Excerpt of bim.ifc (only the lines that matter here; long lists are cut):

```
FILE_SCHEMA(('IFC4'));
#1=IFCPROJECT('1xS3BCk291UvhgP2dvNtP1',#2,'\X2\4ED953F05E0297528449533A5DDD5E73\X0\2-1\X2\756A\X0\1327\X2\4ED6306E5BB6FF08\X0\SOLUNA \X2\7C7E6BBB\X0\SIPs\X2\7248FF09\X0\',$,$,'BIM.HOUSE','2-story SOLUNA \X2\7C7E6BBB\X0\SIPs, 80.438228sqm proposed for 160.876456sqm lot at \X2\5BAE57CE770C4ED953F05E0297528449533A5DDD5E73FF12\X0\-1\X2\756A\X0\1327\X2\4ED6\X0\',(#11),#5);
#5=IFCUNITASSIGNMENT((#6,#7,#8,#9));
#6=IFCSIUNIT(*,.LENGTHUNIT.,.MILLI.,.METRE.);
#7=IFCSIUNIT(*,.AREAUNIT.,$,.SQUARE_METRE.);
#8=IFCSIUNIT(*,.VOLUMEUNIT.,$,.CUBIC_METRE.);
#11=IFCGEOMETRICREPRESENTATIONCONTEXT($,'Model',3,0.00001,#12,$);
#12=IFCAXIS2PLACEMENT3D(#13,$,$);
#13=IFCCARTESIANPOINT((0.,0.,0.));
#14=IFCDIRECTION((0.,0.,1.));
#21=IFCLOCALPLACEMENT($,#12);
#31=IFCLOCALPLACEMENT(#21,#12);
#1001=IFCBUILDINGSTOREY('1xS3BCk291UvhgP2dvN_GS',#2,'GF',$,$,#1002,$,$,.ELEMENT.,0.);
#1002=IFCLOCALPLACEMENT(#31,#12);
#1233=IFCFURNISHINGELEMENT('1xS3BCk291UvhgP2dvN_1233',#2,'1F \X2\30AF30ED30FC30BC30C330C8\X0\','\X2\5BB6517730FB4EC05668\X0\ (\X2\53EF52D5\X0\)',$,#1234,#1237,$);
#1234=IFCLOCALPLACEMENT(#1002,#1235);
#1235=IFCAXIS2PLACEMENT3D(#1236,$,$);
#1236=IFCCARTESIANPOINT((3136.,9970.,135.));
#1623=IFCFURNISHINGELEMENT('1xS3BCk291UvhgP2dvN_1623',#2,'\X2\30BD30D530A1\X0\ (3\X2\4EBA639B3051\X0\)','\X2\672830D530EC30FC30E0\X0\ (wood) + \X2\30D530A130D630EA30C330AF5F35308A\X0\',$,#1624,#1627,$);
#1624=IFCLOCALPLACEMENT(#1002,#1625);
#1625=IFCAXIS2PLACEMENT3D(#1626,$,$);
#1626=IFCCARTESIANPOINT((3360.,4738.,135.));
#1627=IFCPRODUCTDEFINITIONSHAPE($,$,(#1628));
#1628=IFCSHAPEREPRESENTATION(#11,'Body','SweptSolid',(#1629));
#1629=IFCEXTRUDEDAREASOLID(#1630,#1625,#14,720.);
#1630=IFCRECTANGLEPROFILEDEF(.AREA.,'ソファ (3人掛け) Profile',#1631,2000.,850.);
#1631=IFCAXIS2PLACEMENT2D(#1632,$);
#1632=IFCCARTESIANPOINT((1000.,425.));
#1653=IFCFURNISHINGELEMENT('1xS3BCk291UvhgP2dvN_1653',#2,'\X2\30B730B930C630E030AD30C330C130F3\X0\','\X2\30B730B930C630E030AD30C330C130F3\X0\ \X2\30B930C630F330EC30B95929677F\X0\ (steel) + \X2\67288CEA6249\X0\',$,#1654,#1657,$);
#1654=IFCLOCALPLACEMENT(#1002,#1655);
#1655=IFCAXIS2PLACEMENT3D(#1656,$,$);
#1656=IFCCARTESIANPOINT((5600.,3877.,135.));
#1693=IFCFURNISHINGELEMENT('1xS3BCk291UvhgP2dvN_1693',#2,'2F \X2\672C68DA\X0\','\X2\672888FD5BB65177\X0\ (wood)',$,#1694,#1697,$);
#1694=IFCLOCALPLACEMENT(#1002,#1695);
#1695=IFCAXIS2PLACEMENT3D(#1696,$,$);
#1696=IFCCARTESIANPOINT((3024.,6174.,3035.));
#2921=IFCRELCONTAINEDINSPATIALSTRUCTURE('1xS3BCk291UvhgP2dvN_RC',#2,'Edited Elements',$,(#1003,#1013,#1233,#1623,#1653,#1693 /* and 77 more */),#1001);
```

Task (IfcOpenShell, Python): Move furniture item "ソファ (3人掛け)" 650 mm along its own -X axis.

```python
import ifcopenshell
import ifcopenshell.api.geometry
import ifcopenshell.util.placement
import ifcopenshell.util.unit

model = ifcopenshell.open("bim.ifc")
unit_scale = ifcopenshell.util.unit.calculate_unit_scale(model)

item = model.by_guid("1xS3BCk291UvhgP2dvN_1623")
matrix = ifcopenshell.util.placement.get_local_placement(item.ObjectPlacement)
matrix[:3, 3] -= matrix[:3, 0] * 0.65 / unit_scale
ifcopenshell.api.geometry.edit_object_placement(model, product=item, matrix=matrix, is_si=False)

print(ifcopenshell.util.placement.get_local_placement(item.ObjectPlacement).round(3) + 0.0)

model.write("bim_updated.ifc")
```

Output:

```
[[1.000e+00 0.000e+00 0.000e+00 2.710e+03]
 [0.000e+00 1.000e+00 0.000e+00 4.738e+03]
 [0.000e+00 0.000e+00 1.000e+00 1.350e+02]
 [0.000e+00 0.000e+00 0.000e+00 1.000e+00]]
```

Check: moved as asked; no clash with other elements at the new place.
